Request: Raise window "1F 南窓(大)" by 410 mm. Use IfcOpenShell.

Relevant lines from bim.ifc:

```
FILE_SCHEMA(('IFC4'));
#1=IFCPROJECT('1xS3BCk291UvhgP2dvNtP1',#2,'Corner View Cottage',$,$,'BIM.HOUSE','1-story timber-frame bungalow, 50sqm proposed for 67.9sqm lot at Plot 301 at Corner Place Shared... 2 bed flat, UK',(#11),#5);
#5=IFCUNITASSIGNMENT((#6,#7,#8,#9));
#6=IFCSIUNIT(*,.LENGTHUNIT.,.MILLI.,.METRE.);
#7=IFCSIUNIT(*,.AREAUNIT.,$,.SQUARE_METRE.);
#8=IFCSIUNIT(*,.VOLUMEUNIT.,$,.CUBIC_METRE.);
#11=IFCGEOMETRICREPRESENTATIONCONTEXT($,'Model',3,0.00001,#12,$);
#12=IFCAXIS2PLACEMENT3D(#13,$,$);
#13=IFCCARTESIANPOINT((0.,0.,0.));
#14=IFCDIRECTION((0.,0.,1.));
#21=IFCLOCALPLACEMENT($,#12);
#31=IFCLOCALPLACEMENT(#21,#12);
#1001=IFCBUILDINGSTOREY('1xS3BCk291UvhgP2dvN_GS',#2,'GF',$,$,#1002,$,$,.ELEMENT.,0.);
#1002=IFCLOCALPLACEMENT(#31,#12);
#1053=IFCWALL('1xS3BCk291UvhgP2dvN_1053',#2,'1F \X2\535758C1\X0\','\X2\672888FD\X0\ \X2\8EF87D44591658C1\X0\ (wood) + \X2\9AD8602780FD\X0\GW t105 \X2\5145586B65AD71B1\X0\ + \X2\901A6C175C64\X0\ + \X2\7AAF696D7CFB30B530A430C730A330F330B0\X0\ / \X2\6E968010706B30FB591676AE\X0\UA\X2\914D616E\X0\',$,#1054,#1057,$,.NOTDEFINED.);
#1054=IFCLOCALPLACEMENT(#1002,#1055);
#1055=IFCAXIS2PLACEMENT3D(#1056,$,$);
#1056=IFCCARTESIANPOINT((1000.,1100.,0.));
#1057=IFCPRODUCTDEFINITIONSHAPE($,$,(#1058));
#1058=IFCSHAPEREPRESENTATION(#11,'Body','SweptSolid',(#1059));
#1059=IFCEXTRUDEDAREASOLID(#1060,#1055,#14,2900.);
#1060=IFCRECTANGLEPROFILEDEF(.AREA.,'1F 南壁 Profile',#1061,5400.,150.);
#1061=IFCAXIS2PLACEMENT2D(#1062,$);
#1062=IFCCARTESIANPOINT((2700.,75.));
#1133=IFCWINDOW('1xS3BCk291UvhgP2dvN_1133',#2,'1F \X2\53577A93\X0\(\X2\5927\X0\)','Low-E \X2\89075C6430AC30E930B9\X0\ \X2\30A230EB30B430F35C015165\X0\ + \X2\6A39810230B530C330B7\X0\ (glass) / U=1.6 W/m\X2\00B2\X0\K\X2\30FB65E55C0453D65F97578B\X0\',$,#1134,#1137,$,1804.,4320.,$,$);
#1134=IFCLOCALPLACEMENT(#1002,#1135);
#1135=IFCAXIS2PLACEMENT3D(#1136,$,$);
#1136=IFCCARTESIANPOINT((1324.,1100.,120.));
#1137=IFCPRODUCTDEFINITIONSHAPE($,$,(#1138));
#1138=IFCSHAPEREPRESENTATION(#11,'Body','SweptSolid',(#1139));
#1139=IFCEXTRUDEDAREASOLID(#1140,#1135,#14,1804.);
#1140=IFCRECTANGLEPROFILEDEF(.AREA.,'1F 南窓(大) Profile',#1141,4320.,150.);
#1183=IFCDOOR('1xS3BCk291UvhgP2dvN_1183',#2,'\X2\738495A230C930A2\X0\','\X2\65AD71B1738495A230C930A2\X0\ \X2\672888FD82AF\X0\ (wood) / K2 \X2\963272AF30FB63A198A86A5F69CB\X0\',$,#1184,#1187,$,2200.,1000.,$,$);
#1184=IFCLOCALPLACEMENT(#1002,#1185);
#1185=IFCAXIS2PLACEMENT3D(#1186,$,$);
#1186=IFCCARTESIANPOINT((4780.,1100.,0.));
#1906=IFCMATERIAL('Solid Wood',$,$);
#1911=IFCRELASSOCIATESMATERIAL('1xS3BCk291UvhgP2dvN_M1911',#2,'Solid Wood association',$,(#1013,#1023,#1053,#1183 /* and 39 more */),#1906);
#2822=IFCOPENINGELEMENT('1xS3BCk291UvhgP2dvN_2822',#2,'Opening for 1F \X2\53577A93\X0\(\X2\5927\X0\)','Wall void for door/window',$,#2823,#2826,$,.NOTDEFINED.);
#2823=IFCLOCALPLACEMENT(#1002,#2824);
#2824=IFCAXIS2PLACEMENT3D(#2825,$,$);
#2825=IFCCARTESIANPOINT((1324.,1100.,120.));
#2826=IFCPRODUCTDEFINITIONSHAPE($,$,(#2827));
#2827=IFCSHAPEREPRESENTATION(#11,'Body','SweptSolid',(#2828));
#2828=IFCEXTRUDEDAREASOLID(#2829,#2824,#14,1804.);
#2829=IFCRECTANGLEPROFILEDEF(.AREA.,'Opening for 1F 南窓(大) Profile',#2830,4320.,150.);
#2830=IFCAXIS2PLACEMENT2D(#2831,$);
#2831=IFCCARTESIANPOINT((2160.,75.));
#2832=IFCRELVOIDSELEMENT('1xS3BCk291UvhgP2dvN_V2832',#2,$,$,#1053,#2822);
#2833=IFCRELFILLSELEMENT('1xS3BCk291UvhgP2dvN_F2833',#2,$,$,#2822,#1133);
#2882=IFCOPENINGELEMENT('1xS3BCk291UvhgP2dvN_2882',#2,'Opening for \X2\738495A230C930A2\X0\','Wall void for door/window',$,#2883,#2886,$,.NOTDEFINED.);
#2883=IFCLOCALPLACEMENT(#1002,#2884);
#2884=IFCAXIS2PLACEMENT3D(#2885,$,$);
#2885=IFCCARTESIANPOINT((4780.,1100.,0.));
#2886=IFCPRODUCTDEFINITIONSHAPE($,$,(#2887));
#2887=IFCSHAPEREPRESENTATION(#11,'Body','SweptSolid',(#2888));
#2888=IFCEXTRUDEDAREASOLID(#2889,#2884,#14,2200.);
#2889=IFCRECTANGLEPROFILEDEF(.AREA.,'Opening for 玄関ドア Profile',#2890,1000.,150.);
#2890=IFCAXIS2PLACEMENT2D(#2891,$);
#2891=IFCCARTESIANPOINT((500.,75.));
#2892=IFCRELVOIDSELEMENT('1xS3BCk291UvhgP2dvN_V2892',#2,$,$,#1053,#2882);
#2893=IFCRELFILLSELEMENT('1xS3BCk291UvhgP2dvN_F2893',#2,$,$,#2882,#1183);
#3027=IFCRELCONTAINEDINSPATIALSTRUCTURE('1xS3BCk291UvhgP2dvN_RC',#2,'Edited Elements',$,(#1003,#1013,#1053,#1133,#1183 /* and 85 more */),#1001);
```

```python
import numpy as np
import ifcopenshell
import ifcopenshell.api.geometry
import ifcopenshell.util.placement
import ifcopenshell.util.unit

model = ifcopenshell.open("bim.ifc")
unit_scale = ifcopenshell.util.unit.calculate_unit_scale(model)

window = model.by_guid("1xS3BCk291UvhgP2dvN_1133")
opening = window.FillsVoids[0].RelatingOpeningElement
dz = 0.41 / unit_scale

shift = np.array([0.0, 0.0, dz])
# The window is not placed relative to its opening, so move both.
for product in (opening, window):
    matrix = ifcopenshell.util.placement.get_local_placement(product.ObjectPlacement)
    matrix[:3, 3] += shift
    ifcopenshell.api.geometry.edit_object_placement(model, product=product, matrix=matrix, is_si=False)

print(f"moved by {dz * unit_scale:+.3f} m")

model.write("bim_v2.ifc")
```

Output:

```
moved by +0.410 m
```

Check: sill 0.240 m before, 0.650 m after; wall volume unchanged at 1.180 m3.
